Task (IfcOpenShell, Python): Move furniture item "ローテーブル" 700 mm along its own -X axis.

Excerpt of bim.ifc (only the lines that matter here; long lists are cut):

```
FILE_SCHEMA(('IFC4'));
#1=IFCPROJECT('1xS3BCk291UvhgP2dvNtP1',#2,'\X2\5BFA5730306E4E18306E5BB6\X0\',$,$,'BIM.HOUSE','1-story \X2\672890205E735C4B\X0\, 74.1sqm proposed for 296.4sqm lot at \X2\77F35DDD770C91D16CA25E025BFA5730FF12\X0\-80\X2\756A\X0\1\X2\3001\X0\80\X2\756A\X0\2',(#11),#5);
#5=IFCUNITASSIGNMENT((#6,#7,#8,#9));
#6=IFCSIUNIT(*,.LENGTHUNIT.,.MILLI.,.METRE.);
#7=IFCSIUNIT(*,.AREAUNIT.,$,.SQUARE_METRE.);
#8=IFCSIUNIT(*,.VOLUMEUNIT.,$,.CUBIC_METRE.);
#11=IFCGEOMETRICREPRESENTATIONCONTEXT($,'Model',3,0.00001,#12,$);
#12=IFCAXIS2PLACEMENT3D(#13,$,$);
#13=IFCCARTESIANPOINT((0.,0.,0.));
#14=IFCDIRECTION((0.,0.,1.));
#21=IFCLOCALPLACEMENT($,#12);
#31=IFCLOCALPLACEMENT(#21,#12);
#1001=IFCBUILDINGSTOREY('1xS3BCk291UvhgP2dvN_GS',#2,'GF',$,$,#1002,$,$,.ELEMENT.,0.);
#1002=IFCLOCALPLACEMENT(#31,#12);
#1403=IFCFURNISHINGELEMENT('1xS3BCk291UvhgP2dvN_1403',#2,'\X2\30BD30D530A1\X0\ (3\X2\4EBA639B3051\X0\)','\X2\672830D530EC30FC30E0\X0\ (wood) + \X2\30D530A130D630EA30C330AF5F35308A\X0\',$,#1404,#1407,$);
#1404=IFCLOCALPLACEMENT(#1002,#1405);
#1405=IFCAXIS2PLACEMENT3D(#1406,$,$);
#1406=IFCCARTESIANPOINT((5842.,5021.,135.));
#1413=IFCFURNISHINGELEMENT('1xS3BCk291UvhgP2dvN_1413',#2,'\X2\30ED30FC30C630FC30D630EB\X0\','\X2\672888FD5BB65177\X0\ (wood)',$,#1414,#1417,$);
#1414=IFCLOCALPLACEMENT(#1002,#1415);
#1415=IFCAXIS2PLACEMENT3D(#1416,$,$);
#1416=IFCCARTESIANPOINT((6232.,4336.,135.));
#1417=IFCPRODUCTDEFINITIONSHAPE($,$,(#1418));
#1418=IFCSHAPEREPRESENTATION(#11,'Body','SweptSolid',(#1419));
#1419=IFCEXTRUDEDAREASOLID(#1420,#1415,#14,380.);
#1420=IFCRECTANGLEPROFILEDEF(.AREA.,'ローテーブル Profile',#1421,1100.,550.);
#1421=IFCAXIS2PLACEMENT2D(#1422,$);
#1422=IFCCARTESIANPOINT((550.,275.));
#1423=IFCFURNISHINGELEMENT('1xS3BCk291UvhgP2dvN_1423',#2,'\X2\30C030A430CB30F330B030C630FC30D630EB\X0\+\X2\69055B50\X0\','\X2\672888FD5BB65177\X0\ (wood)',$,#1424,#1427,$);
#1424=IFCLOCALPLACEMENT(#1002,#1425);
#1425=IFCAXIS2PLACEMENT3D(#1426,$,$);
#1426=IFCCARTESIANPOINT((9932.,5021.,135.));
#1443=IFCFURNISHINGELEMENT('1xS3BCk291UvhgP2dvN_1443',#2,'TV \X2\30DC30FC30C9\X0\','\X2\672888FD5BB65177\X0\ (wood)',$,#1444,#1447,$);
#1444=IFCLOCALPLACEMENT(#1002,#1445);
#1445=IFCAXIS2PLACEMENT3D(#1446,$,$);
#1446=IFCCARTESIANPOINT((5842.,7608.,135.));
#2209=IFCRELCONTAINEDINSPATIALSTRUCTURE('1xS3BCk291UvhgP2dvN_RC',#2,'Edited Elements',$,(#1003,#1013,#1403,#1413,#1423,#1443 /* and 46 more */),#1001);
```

```python
import ifcopenshell
import ifcopenshell.api.geometry
import ifcopenshell.util.placement
import ifcopenshell.util.unit

model = ifcopenshell.open("bim.ifc")
unit_scale = ifcopenshell.util.unit.calculate_unit_scale(model)

item = model.by_guid("1xS3BCk291UvhgP2dvN_1413")
matrix = ifcopenshell.util.placement.get_local_placement(item.ObjectPlacement)
matrix[:3, 3] -= matrix[:3, 0] * 0.7 / unit_scale
ifcopenshell.api.geometry.edit_object_placement(model, product=item, matrix=matrix, is_si=False)

print(ifcopenshell.util.placement.get_local_placement(item.ObjectPlacement).round(3) + 0.0)

model.write("bim_v2.ifc")
```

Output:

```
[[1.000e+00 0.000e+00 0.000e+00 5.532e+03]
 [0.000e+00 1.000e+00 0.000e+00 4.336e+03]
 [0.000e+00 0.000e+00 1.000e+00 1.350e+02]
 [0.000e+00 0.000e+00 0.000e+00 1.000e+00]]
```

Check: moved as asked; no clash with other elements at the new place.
